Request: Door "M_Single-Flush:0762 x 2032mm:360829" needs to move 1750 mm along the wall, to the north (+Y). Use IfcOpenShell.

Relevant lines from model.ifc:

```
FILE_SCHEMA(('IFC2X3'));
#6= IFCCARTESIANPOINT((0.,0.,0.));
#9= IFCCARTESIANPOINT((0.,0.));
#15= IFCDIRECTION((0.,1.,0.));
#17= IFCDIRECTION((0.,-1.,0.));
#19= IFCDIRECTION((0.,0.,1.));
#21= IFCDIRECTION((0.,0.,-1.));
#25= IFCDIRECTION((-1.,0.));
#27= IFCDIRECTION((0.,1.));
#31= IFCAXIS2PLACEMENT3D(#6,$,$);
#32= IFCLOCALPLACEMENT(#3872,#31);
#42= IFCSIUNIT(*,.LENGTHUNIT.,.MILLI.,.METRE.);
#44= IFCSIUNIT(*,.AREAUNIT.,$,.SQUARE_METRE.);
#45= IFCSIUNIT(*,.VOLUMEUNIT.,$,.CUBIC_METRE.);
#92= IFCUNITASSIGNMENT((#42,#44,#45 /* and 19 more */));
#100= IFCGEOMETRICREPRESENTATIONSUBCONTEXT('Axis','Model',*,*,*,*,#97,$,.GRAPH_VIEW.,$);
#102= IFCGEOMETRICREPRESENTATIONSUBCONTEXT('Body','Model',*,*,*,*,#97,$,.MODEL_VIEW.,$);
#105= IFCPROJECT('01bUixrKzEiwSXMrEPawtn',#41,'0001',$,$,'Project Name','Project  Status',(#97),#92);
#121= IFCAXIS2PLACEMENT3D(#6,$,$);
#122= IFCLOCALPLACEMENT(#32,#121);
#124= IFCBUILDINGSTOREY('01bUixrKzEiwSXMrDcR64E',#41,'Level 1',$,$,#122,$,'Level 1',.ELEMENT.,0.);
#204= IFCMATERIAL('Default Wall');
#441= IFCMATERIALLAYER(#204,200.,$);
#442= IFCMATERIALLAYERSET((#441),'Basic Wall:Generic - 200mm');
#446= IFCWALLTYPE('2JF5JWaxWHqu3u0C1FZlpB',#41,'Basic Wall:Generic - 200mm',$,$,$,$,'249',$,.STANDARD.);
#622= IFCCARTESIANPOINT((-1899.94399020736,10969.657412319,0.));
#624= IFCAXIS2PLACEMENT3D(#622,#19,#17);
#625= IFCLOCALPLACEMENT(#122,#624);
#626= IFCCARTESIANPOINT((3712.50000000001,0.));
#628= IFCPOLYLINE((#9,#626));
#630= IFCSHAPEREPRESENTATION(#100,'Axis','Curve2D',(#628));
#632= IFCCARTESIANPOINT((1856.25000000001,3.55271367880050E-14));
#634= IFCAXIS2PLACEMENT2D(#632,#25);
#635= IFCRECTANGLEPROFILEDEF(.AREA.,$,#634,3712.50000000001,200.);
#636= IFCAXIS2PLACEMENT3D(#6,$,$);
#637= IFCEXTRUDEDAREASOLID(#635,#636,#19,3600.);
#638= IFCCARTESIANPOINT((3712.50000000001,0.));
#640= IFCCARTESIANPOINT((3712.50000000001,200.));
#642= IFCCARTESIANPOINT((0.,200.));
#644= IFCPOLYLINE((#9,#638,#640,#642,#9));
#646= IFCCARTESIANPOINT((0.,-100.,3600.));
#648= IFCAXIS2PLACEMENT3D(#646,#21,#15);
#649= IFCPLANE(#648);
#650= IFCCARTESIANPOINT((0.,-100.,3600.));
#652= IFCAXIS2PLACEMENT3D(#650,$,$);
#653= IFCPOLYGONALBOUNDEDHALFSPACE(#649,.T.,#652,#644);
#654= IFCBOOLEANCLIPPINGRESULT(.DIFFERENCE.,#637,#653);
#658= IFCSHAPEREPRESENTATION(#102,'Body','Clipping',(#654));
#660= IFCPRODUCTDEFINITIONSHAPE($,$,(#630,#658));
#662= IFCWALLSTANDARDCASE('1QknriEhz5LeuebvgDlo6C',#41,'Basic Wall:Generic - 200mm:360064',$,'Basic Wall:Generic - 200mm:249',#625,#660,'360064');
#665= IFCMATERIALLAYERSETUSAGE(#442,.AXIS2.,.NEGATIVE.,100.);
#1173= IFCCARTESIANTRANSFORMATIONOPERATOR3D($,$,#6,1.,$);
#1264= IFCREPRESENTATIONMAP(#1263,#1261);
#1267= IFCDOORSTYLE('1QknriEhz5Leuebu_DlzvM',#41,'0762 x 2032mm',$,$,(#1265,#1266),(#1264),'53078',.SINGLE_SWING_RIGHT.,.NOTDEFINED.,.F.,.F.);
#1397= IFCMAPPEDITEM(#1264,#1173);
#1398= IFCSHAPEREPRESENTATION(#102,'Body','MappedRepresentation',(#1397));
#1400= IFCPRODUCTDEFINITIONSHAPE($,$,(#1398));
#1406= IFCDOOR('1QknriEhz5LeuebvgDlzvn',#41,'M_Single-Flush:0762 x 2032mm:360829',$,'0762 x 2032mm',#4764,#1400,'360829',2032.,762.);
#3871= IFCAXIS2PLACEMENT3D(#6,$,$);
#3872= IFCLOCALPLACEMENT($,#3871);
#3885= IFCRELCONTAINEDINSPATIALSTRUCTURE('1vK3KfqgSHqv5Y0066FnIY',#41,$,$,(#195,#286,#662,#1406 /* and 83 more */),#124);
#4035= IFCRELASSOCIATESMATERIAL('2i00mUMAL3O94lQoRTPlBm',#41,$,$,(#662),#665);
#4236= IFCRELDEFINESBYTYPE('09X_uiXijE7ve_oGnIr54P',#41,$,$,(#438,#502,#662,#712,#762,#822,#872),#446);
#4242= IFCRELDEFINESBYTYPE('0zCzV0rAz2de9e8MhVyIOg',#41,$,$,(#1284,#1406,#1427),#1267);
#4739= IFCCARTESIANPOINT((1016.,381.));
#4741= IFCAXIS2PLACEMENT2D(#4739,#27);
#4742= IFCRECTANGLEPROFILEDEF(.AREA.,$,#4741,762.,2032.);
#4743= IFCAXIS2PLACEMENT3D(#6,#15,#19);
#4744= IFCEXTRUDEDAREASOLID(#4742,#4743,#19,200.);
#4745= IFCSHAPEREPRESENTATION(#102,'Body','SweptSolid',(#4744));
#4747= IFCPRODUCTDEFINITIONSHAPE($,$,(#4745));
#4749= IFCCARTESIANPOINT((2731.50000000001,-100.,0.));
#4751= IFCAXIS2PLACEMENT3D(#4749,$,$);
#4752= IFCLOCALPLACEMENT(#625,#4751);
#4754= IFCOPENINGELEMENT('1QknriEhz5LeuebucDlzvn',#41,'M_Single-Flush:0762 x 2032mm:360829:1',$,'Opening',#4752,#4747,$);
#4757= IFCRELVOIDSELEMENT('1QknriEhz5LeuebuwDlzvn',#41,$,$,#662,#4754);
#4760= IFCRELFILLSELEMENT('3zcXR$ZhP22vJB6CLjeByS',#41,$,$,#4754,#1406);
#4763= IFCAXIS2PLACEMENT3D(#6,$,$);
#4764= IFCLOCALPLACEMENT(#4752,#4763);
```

```python
import ifcopenshell
import ifcopenshell.api.geometry
import ifcopenshell.util.placement
import ifcopenshell.util.unit

model = ifcopenshell.open("model.ifc")
unit_scale = ifcopenshell.util.unit.calculate_unit_scale(model)

door = model.by_guid("1QknriEhz5LeuebvgDlzvn")
opening = door.FillsVoids[0].RelatingOpeningElement
wall = opening.VoidsElements[0].RelatingBuildingElement

wall_matrix = ifcopenshell.util.placement.get_local_placement(wall.ObjectPlacement)
shift = wall_matrix[:3, 0] * -1.75 / unit_scale
before = ifcopenshell.util.placement.get_local_placement(door.ObjectPlacement)[:3, 3].copy()

# The door is placed relative to its opening, so it follows when the opening moves.
matrix = ifcopenshell.util.placement.get_local_placement(opening.ObjectPlacement)
matrix[:3, 3] += shift
ifcopenshell.api.geometry.edit_object_placement(
    model, product=opening, matrix=matrix, is_si=False, should_transform_children=True
)

after = ifcopenshell.util.placement.get_local_placement(door.ObjectPlacement)[:3, 3]
print("door moved by", (after - before).round(3) + 0.0)

model.write("model_v2.ifc")
```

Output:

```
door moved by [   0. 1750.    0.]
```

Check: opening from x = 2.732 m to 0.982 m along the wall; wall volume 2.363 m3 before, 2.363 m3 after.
